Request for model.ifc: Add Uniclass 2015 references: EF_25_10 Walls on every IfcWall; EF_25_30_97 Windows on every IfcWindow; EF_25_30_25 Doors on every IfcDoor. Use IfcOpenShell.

First a look at what the model holds.

```python
import ifcopenshell

model = ifcopenshell.open("model.ifc")
print(model.schema)
print("classifications:", [c.Name for c in model.by_type("IfcClassification")])
for ifc_class in ("IfcDoor", "IfcRoof", "IfcStair", "IfcWall", "IfcWindow"):
    print(ifc_class, len(model.by_type(ifc_class)))
```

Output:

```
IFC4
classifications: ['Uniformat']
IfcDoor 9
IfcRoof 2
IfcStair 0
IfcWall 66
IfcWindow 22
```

```python
import ifcopenshell
import ifcopenshell.api.classification

model = ifcopenshell.open("model.ifc")

system = ifcopenshell.api.classification.add_classification(model, classification="Uniclass 2015")

codes = {
    "IfcWall": ("EF_25_10", "Walls"),
    "IfcWindow": ("EF_25_30_97", "Windows"),
    "IfcDoor": ("EF_25_30_25", "Doors"),
}
for ifc_class, (code, name) in codes.items():
    products = model.by_type(ifc_class)
    ifcopenshell.api.classification.add_reference(
        model, products=products, classification=system, identification=code, name=name
    )
    print(code, len(products))

model.write("model_v2.ifc")
```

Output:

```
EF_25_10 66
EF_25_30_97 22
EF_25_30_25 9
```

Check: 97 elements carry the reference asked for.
